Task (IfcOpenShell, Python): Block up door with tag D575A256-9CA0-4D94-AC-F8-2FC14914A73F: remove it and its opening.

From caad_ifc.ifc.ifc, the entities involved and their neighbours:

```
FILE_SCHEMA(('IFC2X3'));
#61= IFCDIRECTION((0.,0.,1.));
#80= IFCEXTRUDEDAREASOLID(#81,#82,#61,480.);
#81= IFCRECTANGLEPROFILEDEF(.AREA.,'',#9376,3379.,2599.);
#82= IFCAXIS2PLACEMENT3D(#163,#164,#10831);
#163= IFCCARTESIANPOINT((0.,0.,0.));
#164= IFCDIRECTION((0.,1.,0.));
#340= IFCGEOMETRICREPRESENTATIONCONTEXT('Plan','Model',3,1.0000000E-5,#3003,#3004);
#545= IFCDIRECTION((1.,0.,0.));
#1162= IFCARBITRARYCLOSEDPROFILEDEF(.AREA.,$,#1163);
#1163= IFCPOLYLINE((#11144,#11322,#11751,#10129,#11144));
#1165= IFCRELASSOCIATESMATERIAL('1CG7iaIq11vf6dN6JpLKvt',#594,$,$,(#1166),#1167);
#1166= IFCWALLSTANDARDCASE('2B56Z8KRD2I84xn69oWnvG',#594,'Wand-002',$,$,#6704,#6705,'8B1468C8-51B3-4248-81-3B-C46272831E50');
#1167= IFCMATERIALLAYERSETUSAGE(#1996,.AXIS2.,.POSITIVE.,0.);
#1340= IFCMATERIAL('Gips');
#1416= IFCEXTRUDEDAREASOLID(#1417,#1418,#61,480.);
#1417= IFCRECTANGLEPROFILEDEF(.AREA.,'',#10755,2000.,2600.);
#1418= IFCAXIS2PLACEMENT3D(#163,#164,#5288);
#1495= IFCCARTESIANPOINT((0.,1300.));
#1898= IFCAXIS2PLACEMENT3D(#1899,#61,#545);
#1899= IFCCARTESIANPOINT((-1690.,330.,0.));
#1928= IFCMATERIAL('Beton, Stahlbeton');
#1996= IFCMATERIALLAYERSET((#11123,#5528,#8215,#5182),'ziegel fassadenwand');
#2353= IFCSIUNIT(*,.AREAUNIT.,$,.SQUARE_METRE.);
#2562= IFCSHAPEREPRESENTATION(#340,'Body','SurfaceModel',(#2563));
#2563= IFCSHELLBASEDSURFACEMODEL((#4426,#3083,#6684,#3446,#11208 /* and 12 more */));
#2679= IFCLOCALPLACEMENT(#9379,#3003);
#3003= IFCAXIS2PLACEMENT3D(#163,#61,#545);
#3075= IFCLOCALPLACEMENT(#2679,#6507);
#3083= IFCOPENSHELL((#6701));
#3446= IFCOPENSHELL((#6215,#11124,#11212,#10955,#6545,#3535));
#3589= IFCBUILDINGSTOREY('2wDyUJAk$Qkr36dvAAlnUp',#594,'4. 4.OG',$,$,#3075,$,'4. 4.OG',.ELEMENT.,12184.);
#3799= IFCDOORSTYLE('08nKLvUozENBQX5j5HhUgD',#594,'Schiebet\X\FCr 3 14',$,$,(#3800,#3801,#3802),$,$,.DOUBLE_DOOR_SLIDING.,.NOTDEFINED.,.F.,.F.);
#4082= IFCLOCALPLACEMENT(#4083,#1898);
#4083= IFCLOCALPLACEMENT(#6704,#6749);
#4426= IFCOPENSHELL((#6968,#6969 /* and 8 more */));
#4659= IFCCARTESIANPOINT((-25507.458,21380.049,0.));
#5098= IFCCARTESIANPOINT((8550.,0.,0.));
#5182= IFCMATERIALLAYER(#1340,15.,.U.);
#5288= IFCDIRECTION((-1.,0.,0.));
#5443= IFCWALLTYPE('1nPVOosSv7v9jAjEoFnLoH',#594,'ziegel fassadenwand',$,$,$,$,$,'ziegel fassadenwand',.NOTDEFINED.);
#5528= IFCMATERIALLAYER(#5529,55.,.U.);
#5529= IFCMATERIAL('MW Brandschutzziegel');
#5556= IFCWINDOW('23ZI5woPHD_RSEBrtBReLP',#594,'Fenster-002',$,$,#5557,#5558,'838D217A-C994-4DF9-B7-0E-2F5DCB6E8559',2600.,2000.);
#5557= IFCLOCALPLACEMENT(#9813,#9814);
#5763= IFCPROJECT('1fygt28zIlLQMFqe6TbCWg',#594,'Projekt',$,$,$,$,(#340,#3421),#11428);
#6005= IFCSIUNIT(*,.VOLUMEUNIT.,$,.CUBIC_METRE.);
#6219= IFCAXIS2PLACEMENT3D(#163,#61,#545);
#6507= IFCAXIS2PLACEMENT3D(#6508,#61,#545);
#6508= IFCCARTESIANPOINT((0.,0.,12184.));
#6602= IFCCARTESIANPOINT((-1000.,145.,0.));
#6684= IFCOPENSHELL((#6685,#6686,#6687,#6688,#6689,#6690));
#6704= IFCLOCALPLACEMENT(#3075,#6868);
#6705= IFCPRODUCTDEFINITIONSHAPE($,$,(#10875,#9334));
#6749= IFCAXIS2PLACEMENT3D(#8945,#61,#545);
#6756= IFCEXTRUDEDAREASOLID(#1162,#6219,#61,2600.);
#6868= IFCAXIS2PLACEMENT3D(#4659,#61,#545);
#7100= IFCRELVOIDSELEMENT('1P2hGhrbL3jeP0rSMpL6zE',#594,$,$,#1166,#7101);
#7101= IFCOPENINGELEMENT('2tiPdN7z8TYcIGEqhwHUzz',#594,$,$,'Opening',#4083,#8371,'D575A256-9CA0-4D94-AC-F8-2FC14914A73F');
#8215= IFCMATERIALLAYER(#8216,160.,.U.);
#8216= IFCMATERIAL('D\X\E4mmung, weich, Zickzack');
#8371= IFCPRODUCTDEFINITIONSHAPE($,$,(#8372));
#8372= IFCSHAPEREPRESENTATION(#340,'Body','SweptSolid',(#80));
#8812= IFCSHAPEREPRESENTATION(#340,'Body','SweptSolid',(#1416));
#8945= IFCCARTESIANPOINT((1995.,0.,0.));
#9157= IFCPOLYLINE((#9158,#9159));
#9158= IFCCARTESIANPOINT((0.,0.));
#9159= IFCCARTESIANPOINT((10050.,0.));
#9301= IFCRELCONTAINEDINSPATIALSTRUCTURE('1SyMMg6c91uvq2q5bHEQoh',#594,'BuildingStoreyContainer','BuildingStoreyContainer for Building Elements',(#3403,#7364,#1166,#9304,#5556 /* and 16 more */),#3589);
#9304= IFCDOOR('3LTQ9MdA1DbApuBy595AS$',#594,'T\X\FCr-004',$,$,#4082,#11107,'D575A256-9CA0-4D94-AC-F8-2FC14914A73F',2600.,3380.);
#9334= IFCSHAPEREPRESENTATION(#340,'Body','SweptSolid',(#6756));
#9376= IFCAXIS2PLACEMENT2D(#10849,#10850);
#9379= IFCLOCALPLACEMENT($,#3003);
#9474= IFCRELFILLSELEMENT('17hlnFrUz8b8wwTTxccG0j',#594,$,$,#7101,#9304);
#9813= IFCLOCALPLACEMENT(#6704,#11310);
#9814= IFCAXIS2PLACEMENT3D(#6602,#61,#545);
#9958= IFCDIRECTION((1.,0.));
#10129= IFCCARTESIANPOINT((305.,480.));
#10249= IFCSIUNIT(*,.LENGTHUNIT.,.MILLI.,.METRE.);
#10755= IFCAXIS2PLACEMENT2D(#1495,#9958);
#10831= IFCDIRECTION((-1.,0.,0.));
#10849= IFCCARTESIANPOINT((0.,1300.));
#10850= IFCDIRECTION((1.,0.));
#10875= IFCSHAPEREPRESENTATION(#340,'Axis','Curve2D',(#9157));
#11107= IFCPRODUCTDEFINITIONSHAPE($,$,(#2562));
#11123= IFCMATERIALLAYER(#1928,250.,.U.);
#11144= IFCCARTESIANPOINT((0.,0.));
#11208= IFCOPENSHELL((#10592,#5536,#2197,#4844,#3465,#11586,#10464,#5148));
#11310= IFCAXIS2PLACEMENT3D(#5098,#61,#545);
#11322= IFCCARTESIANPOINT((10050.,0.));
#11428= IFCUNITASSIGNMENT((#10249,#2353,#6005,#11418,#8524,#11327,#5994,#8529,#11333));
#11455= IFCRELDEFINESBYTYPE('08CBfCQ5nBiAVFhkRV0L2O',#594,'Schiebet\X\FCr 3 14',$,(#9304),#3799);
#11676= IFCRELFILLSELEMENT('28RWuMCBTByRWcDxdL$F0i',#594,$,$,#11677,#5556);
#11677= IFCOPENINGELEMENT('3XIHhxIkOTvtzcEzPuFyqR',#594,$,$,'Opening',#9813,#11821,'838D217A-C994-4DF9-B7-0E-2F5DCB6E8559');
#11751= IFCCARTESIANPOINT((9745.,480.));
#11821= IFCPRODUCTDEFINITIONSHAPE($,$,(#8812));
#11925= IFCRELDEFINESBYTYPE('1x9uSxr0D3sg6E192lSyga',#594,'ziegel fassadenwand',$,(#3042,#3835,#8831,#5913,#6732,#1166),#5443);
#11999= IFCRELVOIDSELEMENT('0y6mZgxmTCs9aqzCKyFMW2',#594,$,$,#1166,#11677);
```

```python
import ifcopenshell
import ifcopenshell.api.feature
import ifcopenshell.api.root
import ifcopenshell.geom
import ifcopenshell.util.shape

model = ifcopenshell.open("caad_ifc.ifc.ifc")
settings = ifcopenshell.geom.settings()


def volume(element):
    """Net volume in cubic metres, openings subtracted."""
    shape = ifcopenshell.geom.create_shape(settings, element)
    return ifcopenshell.util.shape.get_volume(shape.geometry)


door = model.by_guid("3LTQ9MdA1DbApuBy595AS$")
opening = door.FillsVoids[0].RelatingOpeningElement
wall = opening.VoidsElements[0].RelatingBuildingElement
before = volume(wall)

ifcopenshell.api.root.remove_product(model, product=door)
ifcopenshell.api.feature.remove_feature(model, feature=opening)

after = volume(wall)

print(f"wall volume {before:.3f} -> {after:.3f} m3")

model.write("caad_ifc.ifc_rev.ifc")
```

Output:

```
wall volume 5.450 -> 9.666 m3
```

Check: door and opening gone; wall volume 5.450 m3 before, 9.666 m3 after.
